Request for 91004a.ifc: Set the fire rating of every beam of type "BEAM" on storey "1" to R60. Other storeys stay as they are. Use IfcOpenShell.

First a look at what the model holds.

```python
import ifcopenshell
import ifcopenshell.util.element

model = ifcopenshell.open("91004a.ifc")
print(model.schema)
storey = next(s for s in model.by_type("IfcBuildingStorey") if s.Name == "1")
beams = [e for e in ifcopenshell.util.element.get_decomposition(storey) if e.is_a("IfcBeam")]
seen = {}
for e in beams:
    element_type = ifcopenshell.util.element.get_type(e)
    key = (element_type.Name if element_type != e and element_type else None, ifcopenshell.util.element.get_pset(e, "Pset_BeamCommon", "FireRating"))
    seen[key] = seen.get(key, 0) + 1
for (name, value), count in sorted(seen.items(), key=str):
    print(count, "x", name, "|", value)
```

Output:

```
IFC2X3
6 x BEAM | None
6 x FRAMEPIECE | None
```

```python
import ifcopenshell
import ifcopenshell.api.pset
import ifcopenshell.util.element

model = ifcopenshell.open("91004a.ifc")

storey = next(s for s in model.by_type("IfcBuildingStorey") if s.Name == "1")
beams = [e for e in ifcopenshell.util.element.get_decomposition(storey) if e.is_a("IfcBeam")]

count = 0
for e in beams:
    element_type = ifcopenshell.util.element.get_type(e)
    if element_type in (None, e) or element_type.Name != "BEAM":
        continue
    # add_pset returns the element's existing set when there is one.
    pset = ifcopenshell.api.pset.add_pset(model, product=e, name="Pset_BeamCommon")
    ifcopenshell.api.pset.edit_pset(model, pset=pset, properties={"FireRating": "R60"})
    count += 1

print(count, "beams updated")

model.write("91004a_edited.ifc")
```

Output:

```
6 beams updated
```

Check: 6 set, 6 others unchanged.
